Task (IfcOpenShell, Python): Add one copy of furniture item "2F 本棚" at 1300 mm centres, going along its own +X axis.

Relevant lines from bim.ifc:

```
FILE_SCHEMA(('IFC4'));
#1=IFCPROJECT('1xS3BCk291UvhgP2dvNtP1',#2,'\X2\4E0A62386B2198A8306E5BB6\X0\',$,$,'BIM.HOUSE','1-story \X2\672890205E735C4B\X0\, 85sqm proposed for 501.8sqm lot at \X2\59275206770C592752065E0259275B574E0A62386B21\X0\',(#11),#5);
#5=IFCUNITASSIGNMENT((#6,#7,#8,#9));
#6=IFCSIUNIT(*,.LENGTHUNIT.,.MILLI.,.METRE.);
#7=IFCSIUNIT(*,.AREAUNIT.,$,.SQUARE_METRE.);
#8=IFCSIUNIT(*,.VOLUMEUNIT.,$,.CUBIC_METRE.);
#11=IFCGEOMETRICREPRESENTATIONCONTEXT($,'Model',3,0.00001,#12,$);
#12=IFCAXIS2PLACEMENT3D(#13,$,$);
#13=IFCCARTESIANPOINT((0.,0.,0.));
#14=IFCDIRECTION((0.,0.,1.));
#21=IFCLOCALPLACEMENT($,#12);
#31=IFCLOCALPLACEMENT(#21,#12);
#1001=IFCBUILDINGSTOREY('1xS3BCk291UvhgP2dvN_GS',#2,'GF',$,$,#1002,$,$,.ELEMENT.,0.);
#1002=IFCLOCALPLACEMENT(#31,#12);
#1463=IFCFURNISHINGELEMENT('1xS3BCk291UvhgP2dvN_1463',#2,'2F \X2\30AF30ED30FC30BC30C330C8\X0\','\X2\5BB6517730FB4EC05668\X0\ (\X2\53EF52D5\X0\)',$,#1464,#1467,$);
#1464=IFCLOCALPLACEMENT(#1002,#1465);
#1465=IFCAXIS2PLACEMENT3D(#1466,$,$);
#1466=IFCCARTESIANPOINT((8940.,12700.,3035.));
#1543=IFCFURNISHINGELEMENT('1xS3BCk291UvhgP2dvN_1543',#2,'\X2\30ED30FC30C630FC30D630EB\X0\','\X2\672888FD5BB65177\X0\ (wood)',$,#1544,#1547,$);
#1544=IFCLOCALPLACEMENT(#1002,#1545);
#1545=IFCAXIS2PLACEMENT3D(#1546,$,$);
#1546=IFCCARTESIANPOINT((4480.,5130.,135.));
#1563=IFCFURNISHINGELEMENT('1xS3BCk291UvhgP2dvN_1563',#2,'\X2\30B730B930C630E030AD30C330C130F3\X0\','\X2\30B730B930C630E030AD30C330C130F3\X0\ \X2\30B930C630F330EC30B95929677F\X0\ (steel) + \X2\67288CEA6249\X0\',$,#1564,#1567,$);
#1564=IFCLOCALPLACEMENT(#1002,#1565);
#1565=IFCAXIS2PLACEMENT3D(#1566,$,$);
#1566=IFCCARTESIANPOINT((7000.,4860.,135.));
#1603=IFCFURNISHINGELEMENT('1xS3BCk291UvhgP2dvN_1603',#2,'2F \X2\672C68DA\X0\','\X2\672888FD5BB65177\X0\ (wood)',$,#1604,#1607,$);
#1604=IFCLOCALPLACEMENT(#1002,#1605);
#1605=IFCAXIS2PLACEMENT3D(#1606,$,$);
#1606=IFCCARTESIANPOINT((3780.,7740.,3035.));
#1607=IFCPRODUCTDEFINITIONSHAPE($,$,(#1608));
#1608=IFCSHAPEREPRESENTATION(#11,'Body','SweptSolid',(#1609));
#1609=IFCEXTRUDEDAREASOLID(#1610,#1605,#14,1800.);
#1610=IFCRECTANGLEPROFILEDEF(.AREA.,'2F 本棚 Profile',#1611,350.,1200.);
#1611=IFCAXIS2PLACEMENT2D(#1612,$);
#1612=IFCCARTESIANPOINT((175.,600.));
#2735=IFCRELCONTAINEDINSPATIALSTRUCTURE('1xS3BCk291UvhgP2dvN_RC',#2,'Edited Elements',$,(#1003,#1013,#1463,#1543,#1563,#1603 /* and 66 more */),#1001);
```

```python
import ifcopenshell
import ifcopenshell.api.geometry
import ifcopenshell.api.root
import ifcopenshell.util.element
import ifcopenshell.util.placement

model = ifcopenshell.open("bim.ifc")


def reuse_history(source, copy):
    """copy_class also copies each property set's owner history, people and application; keep the originals."""
    for rel in copy.IsDefinedBy:
        if rel.is_a("IfcRelDefinesByProperties") and (history := rel.RelatingPropertyDefinition.OwnerHistory):
            rel.RelatingPropertyDefinition.OwnerHistory = source.OwnerHistory
            ifcopenshell.util.element.remove_deep2(model, history)


source = model.by_guid("1xS3BCk291UvhgP2dvN_1603")
base = ifcopenshell.util.placement.get_local_placement(source.ObjectPlacement)
step = base[:3, 0] * 1300.0

for i in range(1, 2):
    copy = ifcopenshell.api.root.copy_class(model, product=source)
    copy.Representation = ifcopenshell.util.element.copy_deep(
        model, source.Representation, exclude=["IfcGeometricRepresentationContext", "IfcRepresentationMap"]
    )
    reuse_history(source, copy)
    matrix = base.copy()
    matrix[:3, 3] += i * step
    print("added at", matrix[:3, 3].round(3) + 0.0)
    ifcopenshell.api.geometry.edit_object_placement(model, product=copy, matrix=matrix, is_si=False)

model.write("bim_v2.ifc")
```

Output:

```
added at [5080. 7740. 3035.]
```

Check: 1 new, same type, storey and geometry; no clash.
